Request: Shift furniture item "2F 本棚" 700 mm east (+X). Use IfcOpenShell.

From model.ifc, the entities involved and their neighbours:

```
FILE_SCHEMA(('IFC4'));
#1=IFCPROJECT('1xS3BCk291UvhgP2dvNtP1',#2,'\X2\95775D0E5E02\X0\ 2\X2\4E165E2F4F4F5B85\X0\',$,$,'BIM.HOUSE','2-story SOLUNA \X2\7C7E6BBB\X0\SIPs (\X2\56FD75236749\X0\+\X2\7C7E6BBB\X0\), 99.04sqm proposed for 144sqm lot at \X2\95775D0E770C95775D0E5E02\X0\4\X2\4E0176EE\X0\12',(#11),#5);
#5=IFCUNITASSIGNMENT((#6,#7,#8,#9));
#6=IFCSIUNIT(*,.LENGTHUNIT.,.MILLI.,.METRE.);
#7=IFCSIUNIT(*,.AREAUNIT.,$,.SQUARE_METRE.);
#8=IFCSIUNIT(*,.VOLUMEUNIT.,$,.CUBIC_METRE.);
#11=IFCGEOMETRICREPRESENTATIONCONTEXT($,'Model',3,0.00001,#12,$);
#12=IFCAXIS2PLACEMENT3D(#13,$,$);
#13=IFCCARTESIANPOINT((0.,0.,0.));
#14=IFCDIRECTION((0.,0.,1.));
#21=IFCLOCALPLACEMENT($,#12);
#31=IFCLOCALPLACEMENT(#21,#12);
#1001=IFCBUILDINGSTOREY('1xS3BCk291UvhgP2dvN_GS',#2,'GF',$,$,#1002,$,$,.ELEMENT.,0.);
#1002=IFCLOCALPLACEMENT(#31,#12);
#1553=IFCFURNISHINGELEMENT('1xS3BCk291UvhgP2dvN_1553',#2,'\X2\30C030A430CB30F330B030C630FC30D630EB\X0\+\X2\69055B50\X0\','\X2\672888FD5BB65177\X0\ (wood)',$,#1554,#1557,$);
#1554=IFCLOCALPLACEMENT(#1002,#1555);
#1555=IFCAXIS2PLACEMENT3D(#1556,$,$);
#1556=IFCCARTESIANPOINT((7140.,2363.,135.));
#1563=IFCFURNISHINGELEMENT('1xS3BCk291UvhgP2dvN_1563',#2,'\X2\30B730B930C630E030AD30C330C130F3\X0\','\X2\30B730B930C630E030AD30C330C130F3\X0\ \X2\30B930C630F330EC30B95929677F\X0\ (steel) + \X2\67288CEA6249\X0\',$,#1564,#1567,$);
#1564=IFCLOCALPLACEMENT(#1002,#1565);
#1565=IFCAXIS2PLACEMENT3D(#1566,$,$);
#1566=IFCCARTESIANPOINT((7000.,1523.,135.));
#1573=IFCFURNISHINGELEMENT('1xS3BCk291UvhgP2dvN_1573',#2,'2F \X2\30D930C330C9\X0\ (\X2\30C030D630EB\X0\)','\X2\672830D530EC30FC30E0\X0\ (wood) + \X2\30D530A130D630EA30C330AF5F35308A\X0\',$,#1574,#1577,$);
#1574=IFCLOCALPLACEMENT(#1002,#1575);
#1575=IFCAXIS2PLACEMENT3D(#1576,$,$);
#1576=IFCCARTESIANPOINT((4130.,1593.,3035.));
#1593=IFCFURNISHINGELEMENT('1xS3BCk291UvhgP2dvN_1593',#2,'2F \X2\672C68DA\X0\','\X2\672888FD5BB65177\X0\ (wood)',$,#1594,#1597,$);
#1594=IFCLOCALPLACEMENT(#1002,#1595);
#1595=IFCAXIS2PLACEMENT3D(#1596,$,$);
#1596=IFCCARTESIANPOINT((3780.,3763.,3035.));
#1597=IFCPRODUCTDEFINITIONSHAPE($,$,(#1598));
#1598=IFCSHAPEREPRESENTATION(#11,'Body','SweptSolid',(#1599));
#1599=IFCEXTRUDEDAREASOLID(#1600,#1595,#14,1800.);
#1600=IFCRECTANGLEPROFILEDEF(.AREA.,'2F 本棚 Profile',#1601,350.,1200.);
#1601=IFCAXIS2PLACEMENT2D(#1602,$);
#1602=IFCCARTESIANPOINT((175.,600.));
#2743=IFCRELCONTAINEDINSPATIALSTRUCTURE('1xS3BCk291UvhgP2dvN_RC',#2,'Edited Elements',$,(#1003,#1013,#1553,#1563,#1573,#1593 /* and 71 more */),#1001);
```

```python
import ifcopenshell
import ifcopenshell.api.geometry
import ifcopenshell.util.placement

model = ifcopenshell.open("model.ifc")

item = model.by_guid("1xS3BCk291UvhgP2dvN_1593")
matrix = ifcopenshell.util.placement.get_local_placement(item.ObjectPlacement)
matrix[0, 3] += 700.0
ifcopenshell.api.geometry.edit_object_placement(model, product=item, matrix=matrix, is_si=False)

print(ifcopenshell.util.placement.get_local_placement(item.ObjectPlacement).round(3) + 0.0)

model.write("model_rev.ifc")
```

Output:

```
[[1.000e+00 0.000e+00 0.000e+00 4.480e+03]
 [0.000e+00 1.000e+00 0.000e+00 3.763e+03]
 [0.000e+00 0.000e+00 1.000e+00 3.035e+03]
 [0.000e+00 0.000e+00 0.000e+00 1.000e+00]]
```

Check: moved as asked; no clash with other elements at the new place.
